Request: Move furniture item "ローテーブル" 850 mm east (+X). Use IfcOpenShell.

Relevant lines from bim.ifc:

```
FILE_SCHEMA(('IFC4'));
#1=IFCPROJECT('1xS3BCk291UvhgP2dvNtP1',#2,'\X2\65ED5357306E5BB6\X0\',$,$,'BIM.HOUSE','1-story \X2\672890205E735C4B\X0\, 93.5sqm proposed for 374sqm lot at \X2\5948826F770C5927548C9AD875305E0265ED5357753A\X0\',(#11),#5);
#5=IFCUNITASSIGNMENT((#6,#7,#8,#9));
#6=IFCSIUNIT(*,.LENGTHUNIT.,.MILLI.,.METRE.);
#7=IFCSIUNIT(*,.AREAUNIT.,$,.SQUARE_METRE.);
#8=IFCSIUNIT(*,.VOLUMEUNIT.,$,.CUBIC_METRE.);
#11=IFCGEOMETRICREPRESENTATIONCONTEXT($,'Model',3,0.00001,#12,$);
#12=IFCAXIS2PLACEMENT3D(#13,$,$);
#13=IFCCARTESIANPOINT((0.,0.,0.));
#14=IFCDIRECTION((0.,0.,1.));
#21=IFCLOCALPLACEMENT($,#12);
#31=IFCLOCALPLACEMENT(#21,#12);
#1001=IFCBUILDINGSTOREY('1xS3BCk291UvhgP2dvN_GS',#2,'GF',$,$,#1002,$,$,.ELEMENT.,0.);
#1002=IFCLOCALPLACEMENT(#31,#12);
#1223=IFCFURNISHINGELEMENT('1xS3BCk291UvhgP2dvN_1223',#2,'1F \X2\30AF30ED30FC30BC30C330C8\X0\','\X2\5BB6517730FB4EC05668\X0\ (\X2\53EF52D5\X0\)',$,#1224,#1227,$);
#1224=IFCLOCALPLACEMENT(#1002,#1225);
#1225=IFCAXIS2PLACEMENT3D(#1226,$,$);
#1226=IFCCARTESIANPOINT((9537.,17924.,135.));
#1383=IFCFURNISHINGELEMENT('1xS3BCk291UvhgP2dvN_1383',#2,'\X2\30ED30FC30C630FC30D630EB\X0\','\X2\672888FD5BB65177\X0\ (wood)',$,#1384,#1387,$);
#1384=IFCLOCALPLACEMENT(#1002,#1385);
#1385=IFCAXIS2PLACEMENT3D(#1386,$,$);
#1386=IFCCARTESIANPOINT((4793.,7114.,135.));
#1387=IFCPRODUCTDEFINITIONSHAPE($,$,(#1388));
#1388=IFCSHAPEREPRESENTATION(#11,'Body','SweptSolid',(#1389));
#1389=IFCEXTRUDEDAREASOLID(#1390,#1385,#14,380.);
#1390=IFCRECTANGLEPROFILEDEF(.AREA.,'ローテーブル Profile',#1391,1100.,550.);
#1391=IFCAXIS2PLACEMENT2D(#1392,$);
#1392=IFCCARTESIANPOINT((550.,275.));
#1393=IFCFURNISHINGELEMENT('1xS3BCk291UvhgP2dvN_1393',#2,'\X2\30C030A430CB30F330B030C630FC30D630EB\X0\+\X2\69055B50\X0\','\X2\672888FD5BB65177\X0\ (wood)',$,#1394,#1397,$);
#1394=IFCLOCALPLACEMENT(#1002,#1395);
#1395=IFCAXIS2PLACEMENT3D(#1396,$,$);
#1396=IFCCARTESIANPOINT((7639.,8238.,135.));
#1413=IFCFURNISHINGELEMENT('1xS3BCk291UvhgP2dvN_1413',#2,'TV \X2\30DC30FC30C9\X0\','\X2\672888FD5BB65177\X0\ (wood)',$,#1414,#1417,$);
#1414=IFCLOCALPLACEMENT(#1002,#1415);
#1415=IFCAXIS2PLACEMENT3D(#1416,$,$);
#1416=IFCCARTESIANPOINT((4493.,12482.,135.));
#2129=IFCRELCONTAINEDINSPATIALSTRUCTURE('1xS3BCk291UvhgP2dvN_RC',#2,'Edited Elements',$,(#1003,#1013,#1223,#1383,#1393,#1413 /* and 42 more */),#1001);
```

```python
import ifcopenshell
import ifcopenshell.api.geometry
import ifcopenshell.util.placement

model = ifcopenshell.open("bim.ifc")

item = model.by_guid("1xS3BCk291UvhgP2dvN_1383")
matrix = ifcopenshell.util.placement.get_local_placement(item.ObjectPlacement)
matrix[0, 3] += 850.0
ifcopenshell.api.geometry.edit_object_placement(model, product=item, matrix=matrix, is_si=False)

print(ifcopenshell.util.placement.get_local_placement(item.ObjectPlacement).round(3) + 0.0)

model.write("bim_updated.ifc")
```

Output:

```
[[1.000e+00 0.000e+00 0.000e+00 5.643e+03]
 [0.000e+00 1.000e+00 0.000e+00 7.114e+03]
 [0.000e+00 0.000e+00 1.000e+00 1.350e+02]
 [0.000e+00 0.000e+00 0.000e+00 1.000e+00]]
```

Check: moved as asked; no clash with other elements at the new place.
